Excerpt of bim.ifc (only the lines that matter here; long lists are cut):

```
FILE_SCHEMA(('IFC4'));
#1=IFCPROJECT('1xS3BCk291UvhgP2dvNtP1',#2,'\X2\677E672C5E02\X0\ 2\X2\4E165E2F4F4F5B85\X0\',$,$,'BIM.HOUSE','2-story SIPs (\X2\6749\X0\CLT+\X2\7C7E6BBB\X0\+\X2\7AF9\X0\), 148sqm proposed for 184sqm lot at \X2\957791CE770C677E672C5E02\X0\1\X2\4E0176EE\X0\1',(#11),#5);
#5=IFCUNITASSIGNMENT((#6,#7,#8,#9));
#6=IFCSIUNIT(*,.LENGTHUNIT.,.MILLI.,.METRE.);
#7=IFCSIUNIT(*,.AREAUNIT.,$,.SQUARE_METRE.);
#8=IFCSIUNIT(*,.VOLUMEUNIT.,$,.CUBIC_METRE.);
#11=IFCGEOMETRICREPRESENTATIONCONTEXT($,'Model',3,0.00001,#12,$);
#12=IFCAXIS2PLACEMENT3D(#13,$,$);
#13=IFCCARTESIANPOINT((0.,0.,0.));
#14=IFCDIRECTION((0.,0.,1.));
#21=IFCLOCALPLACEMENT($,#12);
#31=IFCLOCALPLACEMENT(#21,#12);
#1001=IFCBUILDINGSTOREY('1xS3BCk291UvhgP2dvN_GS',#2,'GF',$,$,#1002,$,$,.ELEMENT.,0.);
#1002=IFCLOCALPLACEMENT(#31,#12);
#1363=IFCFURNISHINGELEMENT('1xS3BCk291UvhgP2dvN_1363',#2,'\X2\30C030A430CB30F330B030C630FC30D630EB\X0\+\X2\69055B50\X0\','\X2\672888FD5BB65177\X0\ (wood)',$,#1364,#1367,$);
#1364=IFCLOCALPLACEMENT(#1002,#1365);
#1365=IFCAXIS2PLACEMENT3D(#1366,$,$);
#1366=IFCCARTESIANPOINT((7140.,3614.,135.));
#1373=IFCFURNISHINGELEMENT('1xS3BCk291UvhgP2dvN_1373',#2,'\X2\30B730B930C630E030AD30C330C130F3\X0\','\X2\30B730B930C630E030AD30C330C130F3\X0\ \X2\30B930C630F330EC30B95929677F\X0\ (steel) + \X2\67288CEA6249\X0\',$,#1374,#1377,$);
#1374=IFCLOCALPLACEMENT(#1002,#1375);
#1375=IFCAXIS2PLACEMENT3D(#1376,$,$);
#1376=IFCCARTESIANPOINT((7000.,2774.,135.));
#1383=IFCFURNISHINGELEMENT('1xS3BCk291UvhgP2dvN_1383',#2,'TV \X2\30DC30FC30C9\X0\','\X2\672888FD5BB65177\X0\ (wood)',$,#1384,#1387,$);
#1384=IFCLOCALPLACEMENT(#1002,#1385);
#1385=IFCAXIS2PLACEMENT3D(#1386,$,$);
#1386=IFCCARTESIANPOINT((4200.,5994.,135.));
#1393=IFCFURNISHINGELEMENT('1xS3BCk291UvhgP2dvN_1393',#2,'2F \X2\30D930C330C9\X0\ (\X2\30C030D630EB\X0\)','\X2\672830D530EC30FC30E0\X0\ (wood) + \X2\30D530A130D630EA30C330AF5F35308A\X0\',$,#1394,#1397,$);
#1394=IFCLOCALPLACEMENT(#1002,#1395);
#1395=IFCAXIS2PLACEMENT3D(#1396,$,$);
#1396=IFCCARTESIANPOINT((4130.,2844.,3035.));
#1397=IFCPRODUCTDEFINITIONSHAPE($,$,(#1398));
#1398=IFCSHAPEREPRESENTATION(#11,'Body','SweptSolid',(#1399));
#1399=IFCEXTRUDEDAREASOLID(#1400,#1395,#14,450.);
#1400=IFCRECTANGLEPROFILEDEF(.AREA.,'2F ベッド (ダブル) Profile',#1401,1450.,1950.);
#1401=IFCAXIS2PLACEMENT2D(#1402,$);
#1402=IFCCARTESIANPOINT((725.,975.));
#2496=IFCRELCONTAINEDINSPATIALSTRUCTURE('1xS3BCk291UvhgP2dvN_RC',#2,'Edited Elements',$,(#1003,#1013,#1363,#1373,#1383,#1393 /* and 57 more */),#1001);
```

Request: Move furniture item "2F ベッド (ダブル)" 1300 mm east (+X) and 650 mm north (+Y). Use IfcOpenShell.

```python
import ifcopenshell
import ifcopenshell.api.geometry
import ifcopenshell.util.placement
import ifcopenshell.util.unit

model = ifcopenshell.open("bim.ifc")
unit_scale = ifcopenshell.util.unit.calculate_unit_scale(model)

item = model.by_guid("1xS3BCk291UvhgP2dvN_1393")
matrix = ifcopenshell.util.placement.get_local_placement(item.ObjectPlacement)
matrix[0, 3] += 1.3 / unit_scale
matrix[1, 3] += 0.65 / unit_scale
ifcopenshell.api.geometry.edit_object_placement(model, product=item, matrix=matrix, is_si=False)

print(ifcopenshell.util.placement.get_local_placement(item.ObjectPlacement).round(3) + 0.0)

model.write("bim_rev.ifc")
```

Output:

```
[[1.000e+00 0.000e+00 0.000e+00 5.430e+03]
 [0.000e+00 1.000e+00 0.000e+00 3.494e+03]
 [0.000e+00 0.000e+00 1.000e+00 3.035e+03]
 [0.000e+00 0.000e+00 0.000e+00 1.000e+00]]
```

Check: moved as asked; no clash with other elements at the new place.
